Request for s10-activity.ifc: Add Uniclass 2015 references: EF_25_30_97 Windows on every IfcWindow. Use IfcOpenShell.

First a look at what the model holds.

```python
import ifcopenshell

model = ifcopenshell.open("s10-activity.ifc")
print(model.schema)
print("classifications:", [c.Name for c in model.by_type("IfcClassification")])
for ifc_class in ("IfcDoor", "IfcRoof", "IfcStair", "IfcWall", "IfcWindow"):
    print(ifc_class, len(model.by_type(ifc_class)))
```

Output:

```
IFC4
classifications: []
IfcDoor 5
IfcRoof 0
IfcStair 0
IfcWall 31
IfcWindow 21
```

```python
import ifcopenshell
import ifcopenshell.api.classification

model = ifcopenshell.open("s10-activity.ifc")

system = ifcopenshell.api.classification.add_classification(model, classification="Uniclass 2015")

codes = {
    "IfcWindow": ("EF_25_30_97", "Windows"),
}
for ifc_class, (code, name) in codes.items():
    products = model.by_type(ifc_class)
    ifcopenshell.api.classification.add_reference(
        model, products=products, classification=system, identification=code, name=name
    )
    print(code, len(products))

model.write("s10-activity_v2.ifc")
```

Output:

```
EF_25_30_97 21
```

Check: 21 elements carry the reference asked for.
